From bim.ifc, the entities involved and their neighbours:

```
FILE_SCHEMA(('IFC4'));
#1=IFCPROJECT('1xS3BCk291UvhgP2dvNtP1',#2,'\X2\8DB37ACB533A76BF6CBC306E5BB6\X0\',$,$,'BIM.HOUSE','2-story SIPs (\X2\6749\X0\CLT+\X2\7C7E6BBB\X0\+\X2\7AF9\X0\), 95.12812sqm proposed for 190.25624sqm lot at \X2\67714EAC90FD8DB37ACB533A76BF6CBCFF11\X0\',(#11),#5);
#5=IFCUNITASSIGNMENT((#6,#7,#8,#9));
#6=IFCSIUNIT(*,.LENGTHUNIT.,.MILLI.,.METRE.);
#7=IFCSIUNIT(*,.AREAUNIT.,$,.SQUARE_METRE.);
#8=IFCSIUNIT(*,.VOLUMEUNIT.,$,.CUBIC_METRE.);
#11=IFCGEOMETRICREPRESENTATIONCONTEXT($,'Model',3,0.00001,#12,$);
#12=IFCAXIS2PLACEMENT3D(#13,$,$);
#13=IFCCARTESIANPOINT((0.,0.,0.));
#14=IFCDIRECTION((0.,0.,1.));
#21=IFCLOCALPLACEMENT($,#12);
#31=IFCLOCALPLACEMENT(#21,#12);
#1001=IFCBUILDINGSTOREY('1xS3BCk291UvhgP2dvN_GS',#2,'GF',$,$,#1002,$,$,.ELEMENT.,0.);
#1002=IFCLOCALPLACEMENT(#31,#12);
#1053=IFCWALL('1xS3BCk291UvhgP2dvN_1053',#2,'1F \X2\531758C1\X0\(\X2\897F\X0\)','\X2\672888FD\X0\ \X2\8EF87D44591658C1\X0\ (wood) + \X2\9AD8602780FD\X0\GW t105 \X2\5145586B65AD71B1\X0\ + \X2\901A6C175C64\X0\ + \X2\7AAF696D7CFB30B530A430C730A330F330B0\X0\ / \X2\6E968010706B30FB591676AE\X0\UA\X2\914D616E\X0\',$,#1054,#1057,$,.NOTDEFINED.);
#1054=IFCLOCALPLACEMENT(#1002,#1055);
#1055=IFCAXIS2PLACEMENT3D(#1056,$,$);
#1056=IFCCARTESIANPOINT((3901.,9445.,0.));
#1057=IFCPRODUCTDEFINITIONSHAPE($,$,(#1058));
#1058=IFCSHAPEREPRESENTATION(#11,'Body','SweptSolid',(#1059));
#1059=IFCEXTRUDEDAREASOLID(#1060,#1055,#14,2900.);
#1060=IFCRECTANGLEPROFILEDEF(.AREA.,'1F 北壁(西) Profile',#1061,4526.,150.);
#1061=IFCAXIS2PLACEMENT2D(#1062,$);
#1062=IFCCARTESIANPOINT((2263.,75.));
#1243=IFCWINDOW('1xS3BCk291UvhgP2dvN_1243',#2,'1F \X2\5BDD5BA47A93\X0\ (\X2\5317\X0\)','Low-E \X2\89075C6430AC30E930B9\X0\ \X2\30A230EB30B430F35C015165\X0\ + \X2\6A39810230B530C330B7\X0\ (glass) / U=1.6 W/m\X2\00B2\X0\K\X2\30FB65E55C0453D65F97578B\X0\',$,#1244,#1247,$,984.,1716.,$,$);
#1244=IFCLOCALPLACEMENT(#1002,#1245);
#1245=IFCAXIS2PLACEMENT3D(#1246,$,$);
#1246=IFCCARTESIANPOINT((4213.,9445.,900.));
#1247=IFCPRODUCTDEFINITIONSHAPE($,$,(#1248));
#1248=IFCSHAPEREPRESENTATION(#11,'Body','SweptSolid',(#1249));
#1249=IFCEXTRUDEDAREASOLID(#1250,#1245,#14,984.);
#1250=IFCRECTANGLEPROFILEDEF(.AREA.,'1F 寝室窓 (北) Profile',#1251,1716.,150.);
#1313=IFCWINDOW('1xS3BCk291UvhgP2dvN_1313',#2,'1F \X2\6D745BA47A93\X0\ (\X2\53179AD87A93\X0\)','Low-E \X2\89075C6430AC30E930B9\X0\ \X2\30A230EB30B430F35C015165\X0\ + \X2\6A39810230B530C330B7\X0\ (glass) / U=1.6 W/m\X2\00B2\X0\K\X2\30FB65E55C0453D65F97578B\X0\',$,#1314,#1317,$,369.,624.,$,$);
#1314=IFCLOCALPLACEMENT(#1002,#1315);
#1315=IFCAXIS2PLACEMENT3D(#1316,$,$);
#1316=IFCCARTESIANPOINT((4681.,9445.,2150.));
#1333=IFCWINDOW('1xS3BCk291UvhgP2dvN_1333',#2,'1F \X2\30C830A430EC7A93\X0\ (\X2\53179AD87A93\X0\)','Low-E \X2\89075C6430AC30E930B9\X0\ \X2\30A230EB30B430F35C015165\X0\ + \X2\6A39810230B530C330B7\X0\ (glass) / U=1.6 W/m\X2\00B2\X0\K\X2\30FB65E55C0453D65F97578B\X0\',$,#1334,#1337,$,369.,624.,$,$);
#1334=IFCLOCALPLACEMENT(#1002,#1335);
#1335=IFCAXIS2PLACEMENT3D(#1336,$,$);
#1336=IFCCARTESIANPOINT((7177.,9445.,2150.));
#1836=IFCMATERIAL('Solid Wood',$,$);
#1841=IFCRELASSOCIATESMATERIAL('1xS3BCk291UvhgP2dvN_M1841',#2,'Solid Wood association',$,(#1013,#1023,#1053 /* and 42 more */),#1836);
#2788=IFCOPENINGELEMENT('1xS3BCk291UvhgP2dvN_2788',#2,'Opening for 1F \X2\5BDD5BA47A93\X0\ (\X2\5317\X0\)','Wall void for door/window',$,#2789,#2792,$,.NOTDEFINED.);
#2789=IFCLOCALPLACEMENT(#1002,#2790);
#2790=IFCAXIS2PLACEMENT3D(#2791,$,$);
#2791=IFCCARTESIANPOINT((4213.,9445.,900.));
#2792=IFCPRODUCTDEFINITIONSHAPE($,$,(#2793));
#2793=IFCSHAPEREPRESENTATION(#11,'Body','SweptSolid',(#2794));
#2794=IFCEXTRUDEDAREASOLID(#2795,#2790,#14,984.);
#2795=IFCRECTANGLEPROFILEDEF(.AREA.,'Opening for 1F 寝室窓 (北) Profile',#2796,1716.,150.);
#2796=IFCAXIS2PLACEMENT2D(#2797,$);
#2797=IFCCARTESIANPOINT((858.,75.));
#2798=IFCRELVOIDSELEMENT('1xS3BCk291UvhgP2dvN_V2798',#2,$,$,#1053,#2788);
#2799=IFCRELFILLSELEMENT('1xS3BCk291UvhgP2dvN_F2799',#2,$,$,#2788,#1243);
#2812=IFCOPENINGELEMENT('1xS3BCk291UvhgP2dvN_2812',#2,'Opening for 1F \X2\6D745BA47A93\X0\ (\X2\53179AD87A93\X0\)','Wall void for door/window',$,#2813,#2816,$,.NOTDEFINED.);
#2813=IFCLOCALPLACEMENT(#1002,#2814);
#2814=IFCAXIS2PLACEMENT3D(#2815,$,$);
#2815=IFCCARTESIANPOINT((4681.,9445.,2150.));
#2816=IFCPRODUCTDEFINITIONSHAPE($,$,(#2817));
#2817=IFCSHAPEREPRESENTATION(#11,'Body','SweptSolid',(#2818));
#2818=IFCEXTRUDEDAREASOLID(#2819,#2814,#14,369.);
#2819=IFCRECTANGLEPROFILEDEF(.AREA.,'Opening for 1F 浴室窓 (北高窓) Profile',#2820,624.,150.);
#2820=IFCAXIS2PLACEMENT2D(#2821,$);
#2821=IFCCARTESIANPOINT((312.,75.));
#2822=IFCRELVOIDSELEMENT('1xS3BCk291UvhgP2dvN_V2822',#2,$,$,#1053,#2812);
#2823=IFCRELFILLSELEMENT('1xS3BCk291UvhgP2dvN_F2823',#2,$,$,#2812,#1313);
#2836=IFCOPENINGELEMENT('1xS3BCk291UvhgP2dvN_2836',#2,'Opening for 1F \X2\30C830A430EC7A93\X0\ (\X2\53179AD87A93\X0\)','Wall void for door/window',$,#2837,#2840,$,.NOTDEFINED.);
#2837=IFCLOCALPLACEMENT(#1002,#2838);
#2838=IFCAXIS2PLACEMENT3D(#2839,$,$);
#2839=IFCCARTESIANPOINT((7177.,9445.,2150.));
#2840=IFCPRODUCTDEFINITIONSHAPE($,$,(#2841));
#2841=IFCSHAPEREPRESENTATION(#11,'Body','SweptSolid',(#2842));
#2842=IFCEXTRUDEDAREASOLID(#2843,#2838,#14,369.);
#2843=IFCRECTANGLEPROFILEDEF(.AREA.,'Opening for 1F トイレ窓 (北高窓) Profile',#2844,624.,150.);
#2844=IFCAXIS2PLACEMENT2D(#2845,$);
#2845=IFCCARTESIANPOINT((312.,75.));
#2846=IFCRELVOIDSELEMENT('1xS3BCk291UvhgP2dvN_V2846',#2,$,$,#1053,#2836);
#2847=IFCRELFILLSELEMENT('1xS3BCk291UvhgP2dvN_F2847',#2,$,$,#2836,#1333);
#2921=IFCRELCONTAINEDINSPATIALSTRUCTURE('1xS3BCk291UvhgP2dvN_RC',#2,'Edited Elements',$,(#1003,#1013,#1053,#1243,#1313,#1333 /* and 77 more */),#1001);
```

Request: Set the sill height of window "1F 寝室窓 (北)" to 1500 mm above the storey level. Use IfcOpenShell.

```python
import numpy as np
import ifcopenshell
import ifcopenshell.api.geometry
import ifcopenshell.geom
import ifcopenshell.util.element
import ifcopenshell.util.placement
import ifcopenshell.util.shape
import ifcopenshell.util.unit

model = ifcopenshell.open("bim.ifc")
unit_scale = ifcopenshell.util.unit.calculate_unit_scale(model)

window = model.by_guid("1xS3BCk291UvhgP2dvN_1243")
opening = window.FillsVoids[0].RelatingOpeningElement
storey = ifcopenshell.util.element.get_container(window, ifc_class="IfcBuildingStorey")
level = ifcopenshell.util.placement.get_local_placement(storey.ObjectPlacement)[2, 3]

# The opening's origin need not be at the sill, so measure its lowest point.
shape = ifcopenshell.geom.create_shape(ifcopenshell.geom.settings(), opening)
bottom = ifcopenshell.util.shape.get_shape_bottom_elevation(shape, shape.geometry) / unit_scale
dz = level + 1.5 / unit_scale - bottom

shift = np.array([0.0, 0.0, dz])
# The window is not placed relative to its opening, so move both.
for product in (opening, window):
    matrix = ifcopenshell.util.placement.get_local_placement(product.ObjectPlacement)
    matrix[:3, 3] += shift
    ifcopenshell.api.geometry.edit_object_placement(model, product=product, matrix=matrix, is_si=False)

print(f"moved by {dz * unit_scale:+.3f} m")

model.write("bim_updated.ifc")
```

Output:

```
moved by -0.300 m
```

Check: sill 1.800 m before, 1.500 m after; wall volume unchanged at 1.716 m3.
